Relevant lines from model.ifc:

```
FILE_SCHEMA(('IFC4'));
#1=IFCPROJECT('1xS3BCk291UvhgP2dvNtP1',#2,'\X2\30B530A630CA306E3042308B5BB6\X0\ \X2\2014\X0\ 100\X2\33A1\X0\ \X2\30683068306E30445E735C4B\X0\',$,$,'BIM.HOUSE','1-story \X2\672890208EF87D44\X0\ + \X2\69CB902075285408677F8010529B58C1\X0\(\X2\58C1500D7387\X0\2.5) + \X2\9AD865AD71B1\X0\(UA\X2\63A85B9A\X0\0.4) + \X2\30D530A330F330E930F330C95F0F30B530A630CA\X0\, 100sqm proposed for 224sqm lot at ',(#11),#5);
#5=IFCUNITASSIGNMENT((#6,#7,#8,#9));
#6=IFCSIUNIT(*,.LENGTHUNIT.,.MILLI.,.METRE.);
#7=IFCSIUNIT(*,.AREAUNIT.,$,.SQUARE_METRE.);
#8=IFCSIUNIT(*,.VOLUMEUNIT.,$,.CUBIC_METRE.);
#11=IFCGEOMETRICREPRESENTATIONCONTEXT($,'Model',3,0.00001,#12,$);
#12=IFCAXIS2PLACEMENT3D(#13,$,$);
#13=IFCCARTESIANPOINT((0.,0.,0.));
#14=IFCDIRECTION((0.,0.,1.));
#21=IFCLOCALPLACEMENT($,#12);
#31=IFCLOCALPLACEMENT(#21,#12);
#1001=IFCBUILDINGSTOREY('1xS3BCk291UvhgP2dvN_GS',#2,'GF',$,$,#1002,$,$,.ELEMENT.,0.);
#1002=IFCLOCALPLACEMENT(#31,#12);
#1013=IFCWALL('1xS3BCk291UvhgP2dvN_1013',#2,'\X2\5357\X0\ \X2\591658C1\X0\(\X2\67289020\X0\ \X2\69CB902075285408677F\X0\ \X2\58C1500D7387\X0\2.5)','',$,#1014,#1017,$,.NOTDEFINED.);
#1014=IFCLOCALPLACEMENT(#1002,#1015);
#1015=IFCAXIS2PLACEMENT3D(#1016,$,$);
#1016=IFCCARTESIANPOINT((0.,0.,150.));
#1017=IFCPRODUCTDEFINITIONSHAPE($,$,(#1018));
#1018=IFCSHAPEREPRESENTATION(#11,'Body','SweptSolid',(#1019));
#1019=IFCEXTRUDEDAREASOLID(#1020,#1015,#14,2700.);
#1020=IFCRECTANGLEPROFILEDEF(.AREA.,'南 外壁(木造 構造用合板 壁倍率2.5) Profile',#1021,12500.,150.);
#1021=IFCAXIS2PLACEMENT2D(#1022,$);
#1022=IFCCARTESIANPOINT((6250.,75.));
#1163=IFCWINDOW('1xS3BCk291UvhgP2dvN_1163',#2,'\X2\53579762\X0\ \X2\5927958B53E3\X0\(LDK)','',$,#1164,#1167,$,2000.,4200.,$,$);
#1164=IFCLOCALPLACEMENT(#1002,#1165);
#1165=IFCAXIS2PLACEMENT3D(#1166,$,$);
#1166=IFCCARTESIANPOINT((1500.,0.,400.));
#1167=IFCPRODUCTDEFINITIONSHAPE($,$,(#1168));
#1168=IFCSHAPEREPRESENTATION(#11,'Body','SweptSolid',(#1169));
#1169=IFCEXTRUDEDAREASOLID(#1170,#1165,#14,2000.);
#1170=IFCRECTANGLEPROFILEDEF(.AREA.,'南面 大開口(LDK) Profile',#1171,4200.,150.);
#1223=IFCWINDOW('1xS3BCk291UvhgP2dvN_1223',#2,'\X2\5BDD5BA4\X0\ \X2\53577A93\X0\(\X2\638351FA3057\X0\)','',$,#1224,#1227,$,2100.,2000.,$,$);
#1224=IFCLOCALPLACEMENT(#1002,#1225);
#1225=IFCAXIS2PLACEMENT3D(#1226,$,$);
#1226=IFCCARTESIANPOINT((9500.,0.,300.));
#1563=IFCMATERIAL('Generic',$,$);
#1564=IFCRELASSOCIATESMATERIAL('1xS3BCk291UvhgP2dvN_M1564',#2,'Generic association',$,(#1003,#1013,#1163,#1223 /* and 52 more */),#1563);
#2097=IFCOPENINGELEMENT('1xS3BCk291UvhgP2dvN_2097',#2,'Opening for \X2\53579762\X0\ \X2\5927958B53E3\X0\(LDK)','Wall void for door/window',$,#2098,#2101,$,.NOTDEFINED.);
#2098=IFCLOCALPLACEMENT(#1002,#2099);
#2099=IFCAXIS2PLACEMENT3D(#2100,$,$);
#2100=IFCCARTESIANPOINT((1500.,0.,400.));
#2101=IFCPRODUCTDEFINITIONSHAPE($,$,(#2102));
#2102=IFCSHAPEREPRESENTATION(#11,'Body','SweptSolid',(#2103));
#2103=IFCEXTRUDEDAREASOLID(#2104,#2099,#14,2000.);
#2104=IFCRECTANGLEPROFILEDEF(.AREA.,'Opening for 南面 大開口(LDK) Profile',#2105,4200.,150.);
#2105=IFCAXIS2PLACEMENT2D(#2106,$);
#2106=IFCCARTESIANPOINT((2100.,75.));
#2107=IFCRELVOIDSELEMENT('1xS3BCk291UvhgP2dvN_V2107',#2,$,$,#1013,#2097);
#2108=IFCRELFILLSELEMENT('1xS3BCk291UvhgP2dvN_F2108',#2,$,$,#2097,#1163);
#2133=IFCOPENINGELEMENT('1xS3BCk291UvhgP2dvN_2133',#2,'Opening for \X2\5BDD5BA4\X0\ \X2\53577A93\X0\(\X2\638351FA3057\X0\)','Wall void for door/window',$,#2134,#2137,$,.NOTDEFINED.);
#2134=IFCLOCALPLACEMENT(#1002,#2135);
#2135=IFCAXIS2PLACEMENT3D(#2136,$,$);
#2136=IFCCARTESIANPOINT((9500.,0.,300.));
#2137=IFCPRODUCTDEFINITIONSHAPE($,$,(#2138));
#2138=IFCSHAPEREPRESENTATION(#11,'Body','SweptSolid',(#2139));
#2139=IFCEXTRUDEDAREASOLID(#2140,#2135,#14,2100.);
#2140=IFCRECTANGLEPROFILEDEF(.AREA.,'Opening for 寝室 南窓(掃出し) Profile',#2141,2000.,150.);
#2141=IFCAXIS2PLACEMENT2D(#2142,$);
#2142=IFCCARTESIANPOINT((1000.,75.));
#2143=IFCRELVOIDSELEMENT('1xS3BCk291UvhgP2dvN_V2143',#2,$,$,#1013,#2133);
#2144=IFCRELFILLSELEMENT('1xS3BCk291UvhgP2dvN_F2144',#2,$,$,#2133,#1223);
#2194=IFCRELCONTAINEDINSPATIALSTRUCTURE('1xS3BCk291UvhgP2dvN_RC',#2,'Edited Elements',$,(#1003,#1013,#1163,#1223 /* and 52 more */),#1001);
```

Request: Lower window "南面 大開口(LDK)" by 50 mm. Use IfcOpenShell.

```python
import numpy as np
import ifcopenshell
import ifcopenshell.api.geometry
import ifcopenshell.util.placement
import ifcopenshell.util.unit

model = ifcopenshell.open("model.ifc")
unit_scale = ifcopenshell.util.unit.calculate_unit_scale(model)

window = model.by_guid("1xS3BCk291UvhgP2dvN_1163")
opening = window.FillsVoids[0].RelatingOpeningElement
dz = -50.0

shift = np.array([0.0, 0.0, dz])
# The window is not placed relative to its opening, so move both.
for product in (opening, window):
    matrix = ifcopenshell.util.placement.get_local_placement(product.ObjectPlacement)
    matrix[:3, 3] += shift
    ifcopenshell.api.geometry.edit_object_placement(model, product=product, matrix=matrix, is_si=False)

print(f"moved by {dz * unit_scale:+.3f} m")

model.write("model_rev.ifc")
```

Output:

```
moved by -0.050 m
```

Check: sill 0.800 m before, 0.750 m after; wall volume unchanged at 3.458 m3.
